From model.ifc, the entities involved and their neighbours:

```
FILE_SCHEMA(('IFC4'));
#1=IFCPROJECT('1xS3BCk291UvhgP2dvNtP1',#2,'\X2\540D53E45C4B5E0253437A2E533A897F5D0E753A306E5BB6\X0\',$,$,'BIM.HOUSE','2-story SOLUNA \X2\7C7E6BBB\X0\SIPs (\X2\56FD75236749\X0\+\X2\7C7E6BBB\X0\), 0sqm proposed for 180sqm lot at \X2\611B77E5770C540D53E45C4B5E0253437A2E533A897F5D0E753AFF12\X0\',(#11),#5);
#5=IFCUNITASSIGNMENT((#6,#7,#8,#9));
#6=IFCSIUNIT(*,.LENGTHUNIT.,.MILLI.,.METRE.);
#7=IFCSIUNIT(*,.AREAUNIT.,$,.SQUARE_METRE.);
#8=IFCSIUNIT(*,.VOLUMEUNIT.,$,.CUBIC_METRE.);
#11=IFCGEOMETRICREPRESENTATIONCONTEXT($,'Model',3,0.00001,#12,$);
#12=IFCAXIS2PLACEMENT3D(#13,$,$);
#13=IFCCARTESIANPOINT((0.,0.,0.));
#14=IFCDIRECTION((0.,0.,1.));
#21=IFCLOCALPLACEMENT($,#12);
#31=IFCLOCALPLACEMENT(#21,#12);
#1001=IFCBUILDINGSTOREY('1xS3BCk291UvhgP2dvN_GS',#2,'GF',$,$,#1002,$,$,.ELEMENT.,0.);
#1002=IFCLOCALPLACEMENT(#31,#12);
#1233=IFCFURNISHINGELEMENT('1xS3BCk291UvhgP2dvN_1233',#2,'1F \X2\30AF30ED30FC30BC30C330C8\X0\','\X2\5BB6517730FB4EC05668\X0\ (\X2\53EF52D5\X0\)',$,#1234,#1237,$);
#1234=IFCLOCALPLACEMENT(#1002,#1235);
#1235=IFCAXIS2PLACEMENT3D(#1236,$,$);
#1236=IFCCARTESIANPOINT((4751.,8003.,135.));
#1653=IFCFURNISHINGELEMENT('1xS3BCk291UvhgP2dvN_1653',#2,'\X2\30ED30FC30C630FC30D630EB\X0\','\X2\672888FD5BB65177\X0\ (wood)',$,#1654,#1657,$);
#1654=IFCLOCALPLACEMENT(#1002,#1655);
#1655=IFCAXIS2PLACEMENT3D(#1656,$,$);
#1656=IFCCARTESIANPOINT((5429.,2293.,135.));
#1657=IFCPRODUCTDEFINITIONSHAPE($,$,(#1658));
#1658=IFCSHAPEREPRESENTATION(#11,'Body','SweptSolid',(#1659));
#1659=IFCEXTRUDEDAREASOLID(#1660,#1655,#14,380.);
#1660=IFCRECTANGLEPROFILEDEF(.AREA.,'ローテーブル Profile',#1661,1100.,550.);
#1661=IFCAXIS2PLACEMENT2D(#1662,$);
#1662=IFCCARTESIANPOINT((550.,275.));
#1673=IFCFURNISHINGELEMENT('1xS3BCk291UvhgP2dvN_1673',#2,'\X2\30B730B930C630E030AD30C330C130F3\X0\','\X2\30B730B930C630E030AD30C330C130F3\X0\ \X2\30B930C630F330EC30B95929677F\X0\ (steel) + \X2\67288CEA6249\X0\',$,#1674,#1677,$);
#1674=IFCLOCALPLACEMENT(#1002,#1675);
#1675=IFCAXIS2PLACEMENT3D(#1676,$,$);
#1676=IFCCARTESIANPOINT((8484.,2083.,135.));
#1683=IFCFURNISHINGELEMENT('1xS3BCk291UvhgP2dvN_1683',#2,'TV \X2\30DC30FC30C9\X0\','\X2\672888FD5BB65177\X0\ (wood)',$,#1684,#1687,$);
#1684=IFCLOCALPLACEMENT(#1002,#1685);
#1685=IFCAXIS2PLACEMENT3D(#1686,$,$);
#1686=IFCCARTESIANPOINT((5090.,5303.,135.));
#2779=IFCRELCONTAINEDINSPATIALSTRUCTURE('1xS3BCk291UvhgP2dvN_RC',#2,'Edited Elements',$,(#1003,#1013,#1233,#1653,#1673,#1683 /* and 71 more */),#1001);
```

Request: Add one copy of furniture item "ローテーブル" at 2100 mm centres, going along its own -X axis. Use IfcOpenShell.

```python
import ifcopenshell
import ifcopenshell.api.geometry
import ifcopenshell.api.root
import ifcopenshell.util.element
import ifcopenshell.util.placement
import ifcopenshell.util.unit

model = ifcopenshell.open("model.ifc")
unit_scale = ifcopenshell.util.unit.calculate_unit_scale(model)


def reuse_history(source, copy):
    """copy_class also copies each property set's owner history, people and application; keep the originals."""
    for rel in copy.IsDefinedBy:
        if rel.is_a("IfcRelDefinesByProperties") and (history := rel.RelatingPropertyDefinition.OwnerHistory):
            rel.RelatingPropertyDefinition.OwnerHistory = source.OwnerHistory
            ifcopenshell.util.element.remove_deep2(model, history)


source = model.by_guid("1xS3BCk291UvhgP2dvN_1653")
base = ifcopenshell.util.placement.get_local_placement(source.ObjectPlacement)
step = -base[:3, 0] * 2.1 / unit_scale

for i in range(1, 2):
    copy = ifcopenshell.api.root.copy_class(model, product=source)
    copy.Representation = ifcopenshell.util.element.copy_deep(
        model, source.Representation, exclude=["IfcGeometricRepresentationContext", "IfcRepresentationMap"]
    )
    reuse_history(source, copy)
    matrix = base.copy()
    matrix[:3, 3] += i * step
    print("added at", matrix[:3, 3].round(3) + 0.0)
    ifcopenshell.api.geometry.edit_object_placement(model, product=copy, matrix=matrix, is_si=False)

model.write("model_edited.ifc")
```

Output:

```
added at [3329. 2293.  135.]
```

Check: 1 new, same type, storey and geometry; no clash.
